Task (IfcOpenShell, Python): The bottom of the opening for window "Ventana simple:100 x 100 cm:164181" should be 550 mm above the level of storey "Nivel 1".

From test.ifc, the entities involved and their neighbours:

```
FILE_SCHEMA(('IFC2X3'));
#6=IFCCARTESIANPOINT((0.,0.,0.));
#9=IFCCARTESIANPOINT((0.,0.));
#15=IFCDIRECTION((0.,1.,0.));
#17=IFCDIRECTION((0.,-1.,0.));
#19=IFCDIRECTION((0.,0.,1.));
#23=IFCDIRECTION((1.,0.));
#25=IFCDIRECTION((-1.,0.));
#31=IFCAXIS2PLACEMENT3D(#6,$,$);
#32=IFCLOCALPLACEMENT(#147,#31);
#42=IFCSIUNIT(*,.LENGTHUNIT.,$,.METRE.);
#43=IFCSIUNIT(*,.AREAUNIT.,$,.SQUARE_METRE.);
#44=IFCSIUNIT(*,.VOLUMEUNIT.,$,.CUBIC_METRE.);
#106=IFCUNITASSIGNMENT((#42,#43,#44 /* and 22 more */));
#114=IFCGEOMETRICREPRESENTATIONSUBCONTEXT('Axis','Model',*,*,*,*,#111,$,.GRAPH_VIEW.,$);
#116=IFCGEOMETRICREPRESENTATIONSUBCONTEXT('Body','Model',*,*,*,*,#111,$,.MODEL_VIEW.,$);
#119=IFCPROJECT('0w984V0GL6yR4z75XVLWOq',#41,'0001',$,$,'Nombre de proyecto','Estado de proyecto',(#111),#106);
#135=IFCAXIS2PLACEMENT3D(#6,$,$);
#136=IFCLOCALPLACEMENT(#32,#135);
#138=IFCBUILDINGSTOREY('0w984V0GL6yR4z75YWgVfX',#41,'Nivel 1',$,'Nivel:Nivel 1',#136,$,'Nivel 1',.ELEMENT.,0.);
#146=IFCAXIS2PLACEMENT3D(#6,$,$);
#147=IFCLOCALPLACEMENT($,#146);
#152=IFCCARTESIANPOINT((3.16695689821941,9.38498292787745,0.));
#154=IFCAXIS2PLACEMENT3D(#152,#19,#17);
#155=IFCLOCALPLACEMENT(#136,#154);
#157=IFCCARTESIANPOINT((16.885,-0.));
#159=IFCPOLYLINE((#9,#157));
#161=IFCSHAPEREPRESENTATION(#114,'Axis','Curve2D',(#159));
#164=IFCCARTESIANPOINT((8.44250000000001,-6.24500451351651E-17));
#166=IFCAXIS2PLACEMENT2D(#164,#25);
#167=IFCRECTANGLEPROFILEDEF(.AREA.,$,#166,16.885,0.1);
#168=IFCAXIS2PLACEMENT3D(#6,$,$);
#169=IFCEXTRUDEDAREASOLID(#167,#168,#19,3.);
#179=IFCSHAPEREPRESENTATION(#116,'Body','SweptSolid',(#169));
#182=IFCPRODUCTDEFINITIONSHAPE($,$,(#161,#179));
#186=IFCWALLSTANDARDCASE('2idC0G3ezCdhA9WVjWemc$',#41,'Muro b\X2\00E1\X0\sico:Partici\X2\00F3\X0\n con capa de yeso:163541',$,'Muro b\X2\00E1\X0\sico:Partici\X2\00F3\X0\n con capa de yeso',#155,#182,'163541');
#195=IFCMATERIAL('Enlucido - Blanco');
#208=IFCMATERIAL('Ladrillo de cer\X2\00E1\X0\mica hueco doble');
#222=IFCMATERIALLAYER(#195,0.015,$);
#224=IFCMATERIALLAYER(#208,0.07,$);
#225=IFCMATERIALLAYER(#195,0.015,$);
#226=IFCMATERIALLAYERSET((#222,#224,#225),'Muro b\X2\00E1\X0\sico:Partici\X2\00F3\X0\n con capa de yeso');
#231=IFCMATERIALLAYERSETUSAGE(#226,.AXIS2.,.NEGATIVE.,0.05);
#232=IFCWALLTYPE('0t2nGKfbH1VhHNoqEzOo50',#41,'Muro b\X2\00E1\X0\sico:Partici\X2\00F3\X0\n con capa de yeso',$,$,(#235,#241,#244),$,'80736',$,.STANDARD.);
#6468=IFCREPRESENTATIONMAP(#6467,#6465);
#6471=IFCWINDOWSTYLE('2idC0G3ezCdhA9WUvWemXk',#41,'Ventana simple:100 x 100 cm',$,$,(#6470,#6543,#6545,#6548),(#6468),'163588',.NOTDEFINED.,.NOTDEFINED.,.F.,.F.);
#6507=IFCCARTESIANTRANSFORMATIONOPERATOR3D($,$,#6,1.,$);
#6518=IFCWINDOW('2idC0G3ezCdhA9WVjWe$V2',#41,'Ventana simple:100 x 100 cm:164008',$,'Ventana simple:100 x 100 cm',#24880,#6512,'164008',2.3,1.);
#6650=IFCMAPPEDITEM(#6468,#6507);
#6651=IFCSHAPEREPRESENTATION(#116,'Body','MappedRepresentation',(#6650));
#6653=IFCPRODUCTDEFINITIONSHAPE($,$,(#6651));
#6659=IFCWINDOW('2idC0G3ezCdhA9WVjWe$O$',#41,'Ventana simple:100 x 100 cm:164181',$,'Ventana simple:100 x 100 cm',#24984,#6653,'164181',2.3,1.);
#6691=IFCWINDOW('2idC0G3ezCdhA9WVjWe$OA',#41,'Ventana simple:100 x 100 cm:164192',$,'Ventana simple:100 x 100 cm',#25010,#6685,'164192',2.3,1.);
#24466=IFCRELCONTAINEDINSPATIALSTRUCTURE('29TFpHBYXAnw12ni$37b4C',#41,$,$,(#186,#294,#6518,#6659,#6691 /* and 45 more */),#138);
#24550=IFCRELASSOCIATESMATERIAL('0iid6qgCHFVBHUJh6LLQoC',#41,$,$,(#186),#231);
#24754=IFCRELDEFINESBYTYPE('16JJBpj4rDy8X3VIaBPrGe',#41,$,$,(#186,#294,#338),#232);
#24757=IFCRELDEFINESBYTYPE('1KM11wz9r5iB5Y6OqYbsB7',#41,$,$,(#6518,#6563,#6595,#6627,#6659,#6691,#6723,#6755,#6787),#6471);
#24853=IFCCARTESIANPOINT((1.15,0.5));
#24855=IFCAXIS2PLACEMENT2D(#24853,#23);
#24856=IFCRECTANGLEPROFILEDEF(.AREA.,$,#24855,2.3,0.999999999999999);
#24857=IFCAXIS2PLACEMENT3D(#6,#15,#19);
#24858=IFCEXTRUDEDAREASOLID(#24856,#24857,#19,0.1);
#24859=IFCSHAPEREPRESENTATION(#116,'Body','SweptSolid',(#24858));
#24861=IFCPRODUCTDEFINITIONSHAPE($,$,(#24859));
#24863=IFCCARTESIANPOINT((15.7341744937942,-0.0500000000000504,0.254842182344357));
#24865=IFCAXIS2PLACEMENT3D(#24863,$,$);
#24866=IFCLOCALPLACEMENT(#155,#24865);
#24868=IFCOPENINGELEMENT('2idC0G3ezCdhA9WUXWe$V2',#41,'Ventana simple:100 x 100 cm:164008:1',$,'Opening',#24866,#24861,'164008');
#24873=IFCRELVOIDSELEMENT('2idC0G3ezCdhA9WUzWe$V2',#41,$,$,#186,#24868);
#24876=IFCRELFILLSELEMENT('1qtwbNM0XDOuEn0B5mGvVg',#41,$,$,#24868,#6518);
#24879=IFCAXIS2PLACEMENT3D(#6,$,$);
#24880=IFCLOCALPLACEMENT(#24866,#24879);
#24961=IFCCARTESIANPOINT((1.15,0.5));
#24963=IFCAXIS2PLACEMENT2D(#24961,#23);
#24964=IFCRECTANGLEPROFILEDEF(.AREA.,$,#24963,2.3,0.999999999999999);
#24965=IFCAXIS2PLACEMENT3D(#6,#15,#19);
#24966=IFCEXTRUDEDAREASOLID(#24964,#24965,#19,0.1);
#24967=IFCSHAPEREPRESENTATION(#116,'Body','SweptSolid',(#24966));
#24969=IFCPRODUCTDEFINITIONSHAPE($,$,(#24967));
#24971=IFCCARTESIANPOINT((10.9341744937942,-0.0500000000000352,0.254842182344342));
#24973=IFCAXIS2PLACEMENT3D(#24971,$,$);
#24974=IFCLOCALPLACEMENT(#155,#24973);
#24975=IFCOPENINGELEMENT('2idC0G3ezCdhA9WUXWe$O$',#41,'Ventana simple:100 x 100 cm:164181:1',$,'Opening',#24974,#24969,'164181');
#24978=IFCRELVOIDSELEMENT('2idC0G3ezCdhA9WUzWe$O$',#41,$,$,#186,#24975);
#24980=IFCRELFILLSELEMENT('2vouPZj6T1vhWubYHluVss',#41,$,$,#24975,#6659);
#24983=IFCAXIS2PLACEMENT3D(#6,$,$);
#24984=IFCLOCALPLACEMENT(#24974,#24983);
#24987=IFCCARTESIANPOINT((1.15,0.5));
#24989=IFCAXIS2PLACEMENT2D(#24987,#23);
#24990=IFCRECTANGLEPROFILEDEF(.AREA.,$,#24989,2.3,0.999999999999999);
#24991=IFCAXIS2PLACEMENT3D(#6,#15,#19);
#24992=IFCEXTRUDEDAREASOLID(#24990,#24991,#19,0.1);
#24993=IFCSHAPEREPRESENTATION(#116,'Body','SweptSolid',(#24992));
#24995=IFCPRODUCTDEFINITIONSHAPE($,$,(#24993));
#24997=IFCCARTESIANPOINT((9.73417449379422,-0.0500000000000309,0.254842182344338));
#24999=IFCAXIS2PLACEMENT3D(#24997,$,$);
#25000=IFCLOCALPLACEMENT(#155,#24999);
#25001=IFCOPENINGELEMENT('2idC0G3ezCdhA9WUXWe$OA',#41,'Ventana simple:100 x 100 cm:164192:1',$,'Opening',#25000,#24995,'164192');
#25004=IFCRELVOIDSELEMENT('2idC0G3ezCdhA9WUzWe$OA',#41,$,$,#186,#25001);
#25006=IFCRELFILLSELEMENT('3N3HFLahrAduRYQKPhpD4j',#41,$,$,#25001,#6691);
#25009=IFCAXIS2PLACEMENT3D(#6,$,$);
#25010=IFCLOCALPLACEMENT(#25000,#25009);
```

```python
import numpy as np
import ifcopenshell
import ifcopenshell.api.geometry
import ifcopenshell.geom
import ifcopenshell.util.element
import ifcopenshell.util.placement
import ifcopenshell.util.shape
import ifcopenshell.util.unit

model = ifcopenshell.open("test.ifc")
unit_scale = ifcopenshell.util.unit.calculate_unit_scale(model)

window = model.by_guid("2idC0G3ezCdhA9WVjWe$O$")
opening = window.FillsVoids[0].RelatingOpeningElement
storey = ifcopenshell.util.element.get_container(window, ifc_class="IfcBuildingStorey")
level = ifcopenshell.util.placement.get_local_placement(storey.ObjectPlacement)[2, 3]

# The opening's origin need not be at the sill, so measure its lowest point.
shape = ifcopenshell.geom.create_shape(ifcopenshell.geom.settings(), opening)
bottom = ifcopenshell.util.shape.get_shape_bottom_elevation(shape, shape.geometry) / unit_scale
dz = level + 0.55 / unit_scale - bottom

shift = np.array([0.0, 0.0, dz])
# The window is placed relative to its opening, so it follows when the opening moves.
matrix = ifcopenshell.util.placement.get_local_placement(opening.ObjectPlacement)
matrix[:3, 3] += shift
ifcopenshell.api.geometry.edit_object_placement(
    model, product=opening, matrix=matrix, is_si=False, should_transform_children=True
)

print(f"moved by {dz * unit_scale:+.3f} m")

model.write("test_edited.ifc")
```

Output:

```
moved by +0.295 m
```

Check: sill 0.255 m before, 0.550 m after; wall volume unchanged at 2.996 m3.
